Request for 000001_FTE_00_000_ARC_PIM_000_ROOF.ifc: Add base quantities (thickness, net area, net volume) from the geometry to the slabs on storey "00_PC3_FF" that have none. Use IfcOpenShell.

First a look at what the model holds.

```python
import ifcopenshell
import ifcopenshell.util.element
import ifcopenshell.util.unit

model = ifcopenshell.open("000001_FTE_00_000_ARC_PIM_000_ROOF.ifc")
print(model.schema)
for unit_type in ("LENGTHUNIT", "AREAUNIT", "VOLUMEUNIT"):
    print(unit_type, ifcopenshell.util.unit.calculate_unit_scale(model, unit_type))
storey = next(s for s in model.by_type("IfcBuildingStorey") if s.Name == "00_PC3_FF")
slabs = [e for e in ifcopenshell.util.element.get_decomposition(storey) if e.is_a("IfcSlab")]
for e in sorted(slabs, key=lambda e: e.id()):
    print(e.id(), e.is_a(), e.Name, list(ifcopenshell.util.element.get_psets(e, qtos_only=True)), sep=" | ")
```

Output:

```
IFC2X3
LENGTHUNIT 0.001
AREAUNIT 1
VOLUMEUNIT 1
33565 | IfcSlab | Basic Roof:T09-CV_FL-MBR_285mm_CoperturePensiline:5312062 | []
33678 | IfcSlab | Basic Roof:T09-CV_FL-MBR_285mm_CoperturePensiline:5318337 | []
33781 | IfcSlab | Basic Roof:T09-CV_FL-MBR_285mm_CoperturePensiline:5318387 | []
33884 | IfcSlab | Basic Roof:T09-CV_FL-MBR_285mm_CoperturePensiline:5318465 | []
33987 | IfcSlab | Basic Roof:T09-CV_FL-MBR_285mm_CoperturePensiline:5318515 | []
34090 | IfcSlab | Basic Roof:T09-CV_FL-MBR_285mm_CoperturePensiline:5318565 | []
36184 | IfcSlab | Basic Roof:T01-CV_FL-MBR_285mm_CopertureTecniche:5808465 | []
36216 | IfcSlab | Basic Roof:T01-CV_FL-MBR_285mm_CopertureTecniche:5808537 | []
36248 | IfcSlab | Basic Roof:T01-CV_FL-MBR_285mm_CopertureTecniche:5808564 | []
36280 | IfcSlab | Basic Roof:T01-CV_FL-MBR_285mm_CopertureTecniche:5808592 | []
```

```python
import ifcopenshell
import ifcopenshell.api.pset
import ifcopenshell.geom
import ifcopenshell.util.element
import ifcopenshell.util.shape
import ifcopenshell.util.unit

model = ifcopenshell.open("000001_FTE_00_000_ARC_PIM_000_ROOF.ifc")
unit_scale = ifcopenshell.util.unit.calculate_unit_scale(model)
area_scale = ifcopenshell.util.unit.calculate_unit_scale(model, "AREAUNIT")
volume_scale = ifcopenshell.util.unit.calculate_unit_scale(model, "VOLUMEUNIT")
settings = ifcopenshell.geom.settings()

storey = next(s for s in model.by_type("IfcBuildingStorey") if s.Name == "00_PC3_FF")
slabs = [e for e in ifcopenshell.util.element.get_decomposition(storey) if e.is_a("IfcSlab")]

for e in sorted(slabs, key=lambda e: e.id()):
    if ifcopenshell.util.element.get_psets(e, qtos_only=True, should_inherit=False):
        continue
    # Geometry comes back in metres, in the element's own axes.
    shape = ifcopenshell.geom.create_shape(settings, e)
    values = {
        "Width": ifcopenshell.util.shape.get_z(shape.geometry) / unit_scale,
        "NetArea": ifcopenshell.util.shape.get_footprint_area(shape.geometry) / area_scale,
        "NetVolume": ifcopenshell.util.shape.get_volume(shape.geometry) / volume_scale,
    }
    qto = ifcopenshell.api.pset.add_qto(model, product=e, name="BaseQuantities")
    ifcopenshell.api.pset.edit_qto(model, qto=qto, properties=values)
    print(e.id(), {k: round(v, 3) for k, v in values.items()})

model.write("000001_FTE_00_000_ARC_PIM_000_ROOF_v2.ifc")
```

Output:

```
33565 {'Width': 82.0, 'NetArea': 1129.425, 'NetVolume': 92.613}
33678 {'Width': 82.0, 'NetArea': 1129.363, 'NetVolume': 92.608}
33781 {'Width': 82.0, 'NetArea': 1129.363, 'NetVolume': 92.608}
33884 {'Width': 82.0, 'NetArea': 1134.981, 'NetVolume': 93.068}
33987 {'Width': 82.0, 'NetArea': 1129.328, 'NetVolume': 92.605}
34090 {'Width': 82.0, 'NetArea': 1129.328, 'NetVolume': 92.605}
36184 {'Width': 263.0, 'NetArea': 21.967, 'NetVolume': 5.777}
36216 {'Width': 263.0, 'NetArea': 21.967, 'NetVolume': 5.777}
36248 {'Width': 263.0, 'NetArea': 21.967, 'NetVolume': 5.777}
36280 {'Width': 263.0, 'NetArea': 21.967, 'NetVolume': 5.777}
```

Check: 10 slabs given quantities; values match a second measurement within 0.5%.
